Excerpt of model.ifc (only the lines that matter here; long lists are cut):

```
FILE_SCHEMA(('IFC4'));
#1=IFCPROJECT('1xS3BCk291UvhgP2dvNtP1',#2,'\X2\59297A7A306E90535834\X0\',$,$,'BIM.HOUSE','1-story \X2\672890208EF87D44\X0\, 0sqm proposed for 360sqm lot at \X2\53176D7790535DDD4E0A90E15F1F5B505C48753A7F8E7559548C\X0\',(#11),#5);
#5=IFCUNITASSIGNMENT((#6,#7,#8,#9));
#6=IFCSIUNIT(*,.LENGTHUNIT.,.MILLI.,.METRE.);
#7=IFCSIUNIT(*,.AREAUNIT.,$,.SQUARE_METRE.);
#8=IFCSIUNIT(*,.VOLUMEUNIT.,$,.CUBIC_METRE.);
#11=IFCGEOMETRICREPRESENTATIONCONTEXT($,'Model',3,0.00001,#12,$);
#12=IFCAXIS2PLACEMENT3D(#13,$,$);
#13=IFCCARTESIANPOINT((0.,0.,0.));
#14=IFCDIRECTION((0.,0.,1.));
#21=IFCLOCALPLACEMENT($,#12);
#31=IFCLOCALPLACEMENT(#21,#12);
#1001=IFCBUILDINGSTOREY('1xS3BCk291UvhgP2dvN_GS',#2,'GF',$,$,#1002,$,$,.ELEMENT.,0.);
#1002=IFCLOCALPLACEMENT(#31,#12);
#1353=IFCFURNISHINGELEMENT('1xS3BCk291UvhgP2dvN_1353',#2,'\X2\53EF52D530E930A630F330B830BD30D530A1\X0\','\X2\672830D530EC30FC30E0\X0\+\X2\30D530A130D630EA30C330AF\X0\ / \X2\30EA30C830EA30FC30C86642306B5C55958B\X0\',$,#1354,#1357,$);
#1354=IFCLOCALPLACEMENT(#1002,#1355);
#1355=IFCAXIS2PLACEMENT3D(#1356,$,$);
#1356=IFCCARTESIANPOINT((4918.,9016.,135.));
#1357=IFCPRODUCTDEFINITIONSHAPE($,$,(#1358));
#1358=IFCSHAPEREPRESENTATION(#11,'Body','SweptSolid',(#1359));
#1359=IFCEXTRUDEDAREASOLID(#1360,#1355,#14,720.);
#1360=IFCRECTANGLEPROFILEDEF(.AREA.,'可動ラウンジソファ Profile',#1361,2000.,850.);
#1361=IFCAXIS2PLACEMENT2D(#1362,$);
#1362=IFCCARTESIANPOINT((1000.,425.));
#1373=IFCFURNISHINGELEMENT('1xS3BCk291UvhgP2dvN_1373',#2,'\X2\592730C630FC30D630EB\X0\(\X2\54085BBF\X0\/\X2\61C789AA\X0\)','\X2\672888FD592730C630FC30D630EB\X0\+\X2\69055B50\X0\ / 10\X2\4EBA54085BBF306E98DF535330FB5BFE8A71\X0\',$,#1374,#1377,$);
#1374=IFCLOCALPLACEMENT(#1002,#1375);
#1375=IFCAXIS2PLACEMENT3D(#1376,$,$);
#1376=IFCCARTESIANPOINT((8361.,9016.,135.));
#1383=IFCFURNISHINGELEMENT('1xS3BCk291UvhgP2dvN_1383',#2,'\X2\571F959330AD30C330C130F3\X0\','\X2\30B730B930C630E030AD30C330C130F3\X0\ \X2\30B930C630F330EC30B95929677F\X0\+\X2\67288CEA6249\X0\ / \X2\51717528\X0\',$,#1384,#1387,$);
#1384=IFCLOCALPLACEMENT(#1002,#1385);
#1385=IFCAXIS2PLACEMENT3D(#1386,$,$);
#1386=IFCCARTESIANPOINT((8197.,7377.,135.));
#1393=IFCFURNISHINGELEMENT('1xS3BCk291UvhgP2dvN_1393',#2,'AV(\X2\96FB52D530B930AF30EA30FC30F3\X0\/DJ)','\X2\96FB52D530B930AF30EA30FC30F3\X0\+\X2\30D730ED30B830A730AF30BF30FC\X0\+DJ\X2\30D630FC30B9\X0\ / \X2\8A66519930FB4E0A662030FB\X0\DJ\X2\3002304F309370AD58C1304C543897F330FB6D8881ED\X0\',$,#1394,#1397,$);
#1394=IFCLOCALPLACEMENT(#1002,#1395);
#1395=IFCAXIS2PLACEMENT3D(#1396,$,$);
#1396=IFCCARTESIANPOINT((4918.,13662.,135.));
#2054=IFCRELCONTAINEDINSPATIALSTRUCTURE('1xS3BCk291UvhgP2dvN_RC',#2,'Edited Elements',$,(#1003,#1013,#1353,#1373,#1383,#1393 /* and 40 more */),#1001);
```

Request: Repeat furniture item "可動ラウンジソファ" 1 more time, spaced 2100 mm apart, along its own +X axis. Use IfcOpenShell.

```python
import ifcopenshell
import ifcopenshell.api.geometry
import ifcopenshell.api.root
import ifcopenshell.util.element
import ifcopenshell.util.placement
import ifcopenshell.util.unit

model = ifcopenshell.open("model.ifc")
unit_scale = ifcopenshell.util.unit.calculate_unit_scale(model)


def reuse_history(source, copy):
    """copy_class also copies each property set's owner history, people and application; keep the originals."""
    for rel in copy.IsDefinedBy:
        if rel.is_a("IfcRelDefinesByProperties") and (history := rel.RelatingPropertyDefinition.OwnerHistory):
            rel.RelatingPropertyDefinition.OwnerHistory = source.OwnerHistory
            ifcopenshell.util.element.remove_deep2(model, history)


source = model.by_id(1353)
base = ifcopenshell.util.placement.get_local_placement(source.ObjectPlacement)
step = base[:3, 0] * 2.1 / unit_scale

for i in range(1, 2):
    copy = ifcopenshell.api.root.copy_class(model, product=source)
    copy.Representation = ifcopenshell.util.element.copy_deep(
        model, source.Representation, exclude=["IfcGeometricRepresentationContext", "IfcRepresentationMap"]
    )
    reuse_history(source, copy)
    matrix = base.copy()
    matrix[:3, 3] += i * step
    print("added at", matrix[:3, 3].round(3) + 0.0)
    ifcopenshell.api.geometry.edit_object_placement(model, product=copy, matrix=matrix, is_si=False)

model.write("model-out.ifc")
```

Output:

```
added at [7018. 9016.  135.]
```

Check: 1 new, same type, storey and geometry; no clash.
